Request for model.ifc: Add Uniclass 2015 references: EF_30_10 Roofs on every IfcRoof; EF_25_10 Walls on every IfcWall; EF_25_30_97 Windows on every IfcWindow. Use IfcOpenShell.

First a look at what the model holds.

```python
import ifcopenshell

model = ifcopenshell.open("model.ifc")
print(model.schema)
print("classifications:", [c.Name for c in model.by_type("IfcClassification")])
for ifc_class in ("IfcDoor", "IfcRoof", "IfcStair", "IfcWall", "IfcWindow"):
    print(ifc_class, len(model.by_type(ifc_class)))
```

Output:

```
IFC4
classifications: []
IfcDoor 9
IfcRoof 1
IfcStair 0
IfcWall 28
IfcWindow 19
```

```python
import ifcopenshell
import ifcopenshell.api.classification

model = ifcopenshell.open("model.ifc")

system = ifcopenshell.api.classification.add_classification(model, classification="Uniclass 2015")

codes = {
    "IfcRoof": ("EF_30_10", "Roofs"),
    "IfcWall": ("EF_25_10", "Walls"),
    "IfcWindow": ("EF_25_30_97", "Windows"),
}
for ifc_class, (code, name) in codes.items():
    products = model.by_type(ifc_class)
    ifcopenshell.api.classification.add_reference(
        model, products=products, classification=system, identification=code, name=name
    )
    print(code, len(products))

model.write("model_rev.ifc")
```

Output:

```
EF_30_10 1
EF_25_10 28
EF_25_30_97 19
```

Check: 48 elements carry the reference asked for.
